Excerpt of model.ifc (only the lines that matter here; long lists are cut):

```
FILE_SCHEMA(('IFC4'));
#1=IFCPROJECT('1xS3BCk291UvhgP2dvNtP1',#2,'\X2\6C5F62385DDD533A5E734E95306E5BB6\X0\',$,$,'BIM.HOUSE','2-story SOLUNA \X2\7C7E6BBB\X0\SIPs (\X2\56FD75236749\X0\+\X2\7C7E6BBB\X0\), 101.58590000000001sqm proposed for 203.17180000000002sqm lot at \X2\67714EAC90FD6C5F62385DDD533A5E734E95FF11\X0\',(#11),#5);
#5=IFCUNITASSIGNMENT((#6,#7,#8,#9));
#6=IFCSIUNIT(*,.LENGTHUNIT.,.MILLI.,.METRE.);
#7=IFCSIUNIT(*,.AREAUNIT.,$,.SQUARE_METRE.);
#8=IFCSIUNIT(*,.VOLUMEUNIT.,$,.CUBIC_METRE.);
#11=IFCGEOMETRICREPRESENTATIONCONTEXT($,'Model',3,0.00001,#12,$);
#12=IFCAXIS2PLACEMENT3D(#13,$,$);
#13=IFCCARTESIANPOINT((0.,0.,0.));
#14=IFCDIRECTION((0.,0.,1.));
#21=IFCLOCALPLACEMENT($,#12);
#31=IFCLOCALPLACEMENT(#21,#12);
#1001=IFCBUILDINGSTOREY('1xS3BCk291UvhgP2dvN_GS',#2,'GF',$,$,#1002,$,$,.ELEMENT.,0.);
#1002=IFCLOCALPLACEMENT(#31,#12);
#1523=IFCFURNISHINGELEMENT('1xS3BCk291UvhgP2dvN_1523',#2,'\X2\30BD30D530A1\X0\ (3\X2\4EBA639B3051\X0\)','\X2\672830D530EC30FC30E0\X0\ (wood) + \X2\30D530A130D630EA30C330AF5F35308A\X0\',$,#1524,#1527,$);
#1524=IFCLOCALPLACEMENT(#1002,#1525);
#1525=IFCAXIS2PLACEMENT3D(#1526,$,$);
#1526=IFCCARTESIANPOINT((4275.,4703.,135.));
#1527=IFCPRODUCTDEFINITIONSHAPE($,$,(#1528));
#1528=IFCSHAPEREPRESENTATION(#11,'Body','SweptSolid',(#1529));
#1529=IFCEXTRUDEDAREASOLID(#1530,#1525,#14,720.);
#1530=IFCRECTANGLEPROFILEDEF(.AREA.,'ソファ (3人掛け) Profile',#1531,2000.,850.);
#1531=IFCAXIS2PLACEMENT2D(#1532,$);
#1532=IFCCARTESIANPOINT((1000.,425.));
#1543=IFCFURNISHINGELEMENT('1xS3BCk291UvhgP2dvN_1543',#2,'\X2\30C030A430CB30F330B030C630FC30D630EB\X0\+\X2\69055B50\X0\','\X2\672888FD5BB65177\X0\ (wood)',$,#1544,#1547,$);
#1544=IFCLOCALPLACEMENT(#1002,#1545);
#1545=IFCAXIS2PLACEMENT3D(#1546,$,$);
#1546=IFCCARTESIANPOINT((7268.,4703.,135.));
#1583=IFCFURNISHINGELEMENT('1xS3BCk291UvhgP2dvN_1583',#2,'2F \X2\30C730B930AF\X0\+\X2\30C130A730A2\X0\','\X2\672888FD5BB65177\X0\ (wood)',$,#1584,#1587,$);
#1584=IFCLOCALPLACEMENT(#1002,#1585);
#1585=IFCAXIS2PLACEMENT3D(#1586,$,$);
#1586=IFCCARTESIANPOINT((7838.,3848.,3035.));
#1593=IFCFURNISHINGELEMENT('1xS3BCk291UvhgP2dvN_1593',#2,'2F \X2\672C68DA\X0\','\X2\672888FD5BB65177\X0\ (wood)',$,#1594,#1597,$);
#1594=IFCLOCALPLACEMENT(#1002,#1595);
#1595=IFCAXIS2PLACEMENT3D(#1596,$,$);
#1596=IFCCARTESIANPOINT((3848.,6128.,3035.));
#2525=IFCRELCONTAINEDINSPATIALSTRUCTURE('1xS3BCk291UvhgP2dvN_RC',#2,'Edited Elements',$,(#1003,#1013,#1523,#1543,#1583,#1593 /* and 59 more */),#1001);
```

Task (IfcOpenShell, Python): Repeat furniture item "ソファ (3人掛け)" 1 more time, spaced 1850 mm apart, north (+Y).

```python
import numpy as np
import ifcopenshell
import ifcopenshell.api.geometry
import ifcopenshell.api.root
import ifcopenshell.util.element
import ifcopenshell.util.placement
import ifcopenshell.util.unit

model = ifcopenshell.open("model.ifc")
unit_scale = ifcopenshell.util.unit.calculate_unit_scale(model)


def reuse_history(source, copy):
    """copy_class also copies each property set's owner history, people and application; keep the originals."""
    for rel in copy.IsDefinedBy:
        if rel.is_a("IfcRelDefinesByProperties") and (history := rel.RelatingPropertyDefinition.OwnerHistory):
            rel.RelatingPropertyDefinition.OwnerHistory = source.OwnerHistory
            ifcopenshell.util.element.remove_deep2(model, history)


source = model.by_guid("1xS3BCk291UvhgP2dvN_1523")
base = ifcopenshell.util.placement.get_local_placement(source.ObjectPlacement)
step = np.array([0.0, 1.0, 0.0]) * 1.85 / unit_scale

for i in range(1, 2):
    copy = ifcopenshell.api.root.copy_class(model, product=source)
    copy.Representation = ifcopenshell.util.element.copy_deep(
        model, source.Representation, exclude=["IfcGeometricRepresentationContext", "IfcRepresentationMap"]
    )
    reuse_history(source, copy)
    matrix = base.copy()
    matrix[:3, 3] += i * step
    print("added at", matrix[:3, 3].round(3) + 0.0)
    ifcopenshell.api.geometry.edit_object_placement(model, product=copy, matrix=matrix, is_si=False)

model.write("model_rev.ifc")
```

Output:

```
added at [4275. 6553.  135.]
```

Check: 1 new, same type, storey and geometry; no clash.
